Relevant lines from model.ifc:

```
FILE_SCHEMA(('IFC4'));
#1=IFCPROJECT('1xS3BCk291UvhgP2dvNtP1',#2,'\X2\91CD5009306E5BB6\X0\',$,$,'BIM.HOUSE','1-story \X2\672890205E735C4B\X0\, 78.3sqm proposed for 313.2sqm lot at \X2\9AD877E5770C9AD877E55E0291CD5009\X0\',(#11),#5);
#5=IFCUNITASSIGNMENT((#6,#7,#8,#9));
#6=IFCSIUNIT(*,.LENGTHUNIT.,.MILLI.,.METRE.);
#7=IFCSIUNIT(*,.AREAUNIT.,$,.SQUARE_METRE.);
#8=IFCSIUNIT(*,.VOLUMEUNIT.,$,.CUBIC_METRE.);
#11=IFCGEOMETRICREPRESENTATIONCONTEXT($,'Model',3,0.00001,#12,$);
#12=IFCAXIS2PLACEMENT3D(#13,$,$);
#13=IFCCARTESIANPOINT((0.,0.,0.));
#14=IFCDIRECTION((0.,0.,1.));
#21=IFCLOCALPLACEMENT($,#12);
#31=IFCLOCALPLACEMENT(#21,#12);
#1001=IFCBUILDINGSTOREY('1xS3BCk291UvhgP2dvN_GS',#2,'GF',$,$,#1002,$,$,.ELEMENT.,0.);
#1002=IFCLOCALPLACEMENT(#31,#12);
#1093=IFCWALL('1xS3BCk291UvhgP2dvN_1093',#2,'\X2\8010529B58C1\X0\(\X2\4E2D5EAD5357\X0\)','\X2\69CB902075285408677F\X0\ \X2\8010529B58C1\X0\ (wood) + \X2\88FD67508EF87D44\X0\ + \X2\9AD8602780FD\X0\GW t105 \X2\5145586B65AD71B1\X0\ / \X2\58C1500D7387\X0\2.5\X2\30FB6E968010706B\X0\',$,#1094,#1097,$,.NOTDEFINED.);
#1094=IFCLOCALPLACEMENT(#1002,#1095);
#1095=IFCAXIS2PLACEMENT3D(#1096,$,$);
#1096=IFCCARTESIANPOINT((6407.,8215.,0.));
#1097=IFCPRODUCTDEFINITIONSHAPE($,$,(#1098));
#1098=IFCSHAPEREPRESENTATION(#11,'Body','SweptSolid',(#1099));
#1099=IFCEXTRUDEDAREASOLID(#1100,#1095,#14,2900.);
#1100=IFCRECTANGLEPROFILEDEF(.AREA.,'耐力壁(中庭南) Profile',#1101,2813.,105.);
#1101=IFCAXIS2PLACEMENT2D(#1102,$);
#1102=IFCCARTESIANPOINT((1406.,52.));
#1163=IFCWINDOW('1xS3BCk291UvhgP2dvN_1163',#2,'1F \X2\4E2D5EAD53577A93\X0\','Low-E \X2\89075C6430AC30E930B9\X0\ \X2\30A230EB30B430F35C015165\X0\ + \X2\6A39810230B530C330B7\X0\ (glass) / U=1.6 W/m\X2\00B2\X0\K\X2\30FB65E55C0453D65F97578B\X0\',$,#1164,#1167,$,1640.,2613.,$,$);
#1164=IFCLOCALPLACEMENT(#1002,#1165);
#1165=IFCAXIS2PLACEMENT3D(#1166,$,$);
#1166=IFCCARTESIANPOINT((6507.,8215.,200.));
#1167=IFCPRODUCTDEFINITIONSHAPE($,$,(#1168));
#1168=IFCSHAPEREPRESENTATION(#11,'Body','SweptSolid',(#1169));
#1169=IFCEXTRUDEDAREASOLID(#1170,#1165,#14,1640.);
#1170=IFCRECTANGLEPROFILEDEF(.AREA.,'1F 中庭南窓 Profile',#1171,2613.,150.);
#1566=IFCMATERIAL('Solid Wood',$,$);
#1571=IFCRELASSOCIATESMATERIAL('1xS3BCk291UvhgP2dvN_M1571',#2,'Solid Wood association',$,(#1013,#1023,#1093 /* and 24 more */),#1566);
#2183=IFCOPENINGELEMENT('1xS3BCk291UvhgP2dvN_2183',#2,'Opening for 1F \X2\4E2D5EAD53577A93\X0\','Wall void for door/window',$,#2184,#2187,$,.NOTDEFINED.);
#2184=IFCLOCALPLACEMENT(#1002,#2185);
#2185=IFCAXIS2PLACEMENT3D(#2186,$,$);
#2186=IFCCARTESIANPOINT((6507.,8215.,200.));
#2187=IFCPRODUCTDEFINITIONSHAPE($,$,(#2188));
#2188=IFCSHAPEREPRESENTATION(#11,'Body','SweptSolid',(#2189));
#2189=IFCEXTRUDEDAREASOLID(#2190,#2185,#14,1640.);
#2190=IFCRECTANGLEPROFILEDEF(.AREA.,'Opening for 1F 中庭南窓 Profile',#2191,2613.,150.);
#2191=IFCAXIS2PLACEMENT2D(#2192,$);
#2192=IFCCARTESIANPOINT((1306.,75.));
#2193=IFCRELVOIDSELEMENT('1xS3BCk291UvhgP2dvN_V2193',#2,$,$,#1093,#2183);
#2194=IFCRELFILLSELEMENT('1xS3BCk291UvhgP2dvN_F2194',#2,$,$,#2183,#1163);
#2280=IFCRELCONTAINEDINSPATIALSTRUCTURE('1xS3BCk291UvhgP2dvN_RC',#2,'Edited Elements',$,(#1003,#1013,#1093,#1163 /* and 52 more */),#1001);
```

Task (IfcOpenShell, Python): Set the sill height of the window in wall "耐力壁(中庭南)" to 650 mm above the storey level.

```python
import numpy as np
import ifcopenshell
import ifcopenshell.api.geometry
import ifcopenshell.geom
import ifcopenshell.util.element
import ifcopenshell.util.placement
import ifcopenshell.util.shape
import ifcopenshell.util.unit

model = ifcopenshell.open("model.ifc")
unit_scale = ifcopenshell.util.unit.calculate_unit_scale(model)

window = model.by_guid("1xS3BCk291UvhgP2dvN_1163")
opening = window.FillsVoids[0].RelatingOpeningElement
storey = ifcopenshell.util.element.get_container(window, ifc_class="IfcBuildingStorey")
level = ifcopenshell.util.placement.get_local_placement(storey.ObjectPlacement)[2, 3]

# The opening's origin need not be at the sill, so measure its lowest point.
shape = ifcopenshell.geom.create_shape(ifcopenshell.geom.settings(), opening)
bottom = ifcopenshell.util.shape.get_shape_bottom_elevation(shape, shape.geometry) / unit_scale
dz = level + 0.65 / unit_scale - bottom

shift = np.array([0.0, 0.0, dz])
# The window is not placed relative to its opening, so move both.
for product in (opening, window):
    matrix = ifcopenshell.util.placement.get_local_placement(product.ObjectPlacement)
    matrix[:3, 3] += shift
    ifcopenshell.api.geometry.edit_object_placement(model, product=product, matrix=matrix, is_si=False)

print(f"moved by {dz * unit_scale:+.3f} m")

model.write("model_edited.ifc")
```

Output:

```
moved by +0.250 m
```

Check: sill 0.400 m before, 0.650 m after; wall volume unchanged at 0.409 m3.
